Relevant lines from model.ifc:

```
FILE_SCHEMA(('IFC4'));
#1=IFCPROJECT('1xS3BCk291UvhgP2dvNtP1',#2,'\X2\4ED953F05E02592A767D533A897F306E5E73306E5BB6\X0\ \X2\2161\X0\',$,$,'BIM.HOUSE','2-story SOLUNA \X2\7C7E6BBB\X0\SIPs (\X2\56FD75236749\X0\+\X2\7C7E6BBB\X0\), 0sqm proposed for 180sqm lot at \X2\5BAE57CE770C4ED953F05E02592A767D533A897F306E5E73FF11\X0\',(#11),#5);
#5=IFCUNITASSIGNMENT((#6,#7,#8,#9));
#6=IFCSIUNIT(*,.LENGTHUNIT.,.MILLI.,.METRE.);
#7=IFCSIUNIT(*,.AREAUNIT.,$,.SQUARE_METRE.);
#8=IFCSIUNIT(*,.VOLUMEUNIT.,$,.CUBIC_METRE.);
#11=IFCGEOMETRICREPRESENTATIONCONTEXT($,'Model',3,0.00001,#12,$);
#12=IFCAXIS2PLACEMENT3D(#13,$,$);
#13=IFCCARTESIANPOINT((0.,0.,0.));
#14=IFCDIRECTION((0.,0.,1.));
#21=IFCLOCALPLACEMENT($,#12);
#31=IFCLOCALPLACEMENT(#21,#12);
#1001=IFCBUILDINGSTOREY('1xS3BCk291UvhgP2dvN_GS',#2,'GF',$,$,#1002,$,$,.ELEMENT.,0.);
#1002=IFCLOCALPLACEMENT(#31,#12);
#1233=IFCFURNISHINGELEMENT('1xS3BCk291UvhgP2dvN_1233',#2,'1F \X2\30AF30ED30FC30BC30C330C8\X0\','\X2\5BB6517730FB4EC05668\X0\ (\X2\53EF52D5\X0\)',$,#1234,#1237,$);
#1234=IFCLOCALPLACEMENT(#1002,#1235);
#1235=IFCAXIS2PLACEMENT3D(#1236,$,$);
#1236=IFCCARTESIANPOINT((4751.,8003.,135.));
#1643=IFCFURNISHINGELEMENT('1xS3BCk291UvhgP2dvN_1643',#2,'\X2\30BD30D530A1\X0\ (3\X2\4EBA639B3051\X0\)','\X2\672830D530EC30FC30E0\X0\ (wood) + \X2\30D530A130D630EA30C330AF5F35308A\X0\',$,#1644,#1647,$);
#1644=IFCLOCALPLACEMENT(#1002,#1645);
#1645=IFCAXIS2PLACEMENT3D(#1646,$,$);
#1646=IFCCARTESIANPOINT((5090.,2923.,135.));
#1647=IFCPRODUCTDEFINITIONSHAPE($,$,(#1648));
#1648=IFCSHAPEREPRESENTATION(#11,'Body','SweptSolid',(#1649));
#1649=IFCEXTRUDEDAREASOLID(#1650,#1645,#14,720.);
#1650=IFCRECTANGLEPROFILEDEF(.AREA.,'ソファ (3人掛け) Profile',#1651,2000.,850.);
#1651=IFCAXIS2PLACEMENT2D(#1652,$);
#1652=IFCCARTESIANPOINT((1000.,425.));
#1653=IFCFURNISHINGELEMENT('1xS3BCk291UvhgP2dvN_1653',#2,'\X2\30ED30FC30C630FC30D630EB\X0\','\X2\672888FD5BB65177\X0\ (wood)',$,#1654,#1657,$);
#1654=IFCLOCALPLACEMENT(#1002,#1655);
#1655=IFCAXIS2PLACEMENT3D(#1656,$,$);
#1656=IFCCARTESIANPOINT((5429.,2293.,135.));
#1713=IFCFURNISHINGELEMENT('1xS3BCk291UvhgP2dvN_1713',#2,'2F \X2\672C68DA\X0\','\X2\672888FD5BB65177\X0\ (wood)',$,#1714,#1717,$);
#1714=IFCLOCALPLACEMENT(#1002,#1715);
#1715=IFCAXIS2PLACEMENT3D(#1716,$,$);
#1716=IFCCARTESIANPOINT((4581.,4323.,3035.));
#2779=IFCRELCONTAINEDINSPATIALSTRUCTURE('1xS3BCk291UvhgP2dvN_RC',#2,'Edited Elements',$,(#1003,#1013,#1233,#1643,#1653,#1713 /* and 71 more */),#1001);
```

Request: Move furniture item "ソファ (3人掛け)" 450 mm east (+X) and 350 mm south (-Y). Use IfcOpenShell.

```python
import ifcopenshell
import ifcopenshell.api.geometry
import ifcopenshell.util.placement
import ifcopenshell.util.unit

model = ifcopenshell.open("model.ifc")
unit_scale = ifcopenshell.util.unit.calculate_unit_scale(model)

item = model.by_id(1643)
matrix = ifcopenshell.util.placement.get_local_placement(item.ObjectPlacement)
matrix[0, 3] += 0.45 / unit_scale
matrix[1, 3] -= 0.35 / unit_scale
ifcopenshell.api.geometry.edit_object_placement(model, product=item, matrix=matrix, is_si=False)

print(ifcopenshell.util.placement.get_local_placement(item.ObjectPlacement).round(3) + 0.0)

model.write("model_rev.ifc")
```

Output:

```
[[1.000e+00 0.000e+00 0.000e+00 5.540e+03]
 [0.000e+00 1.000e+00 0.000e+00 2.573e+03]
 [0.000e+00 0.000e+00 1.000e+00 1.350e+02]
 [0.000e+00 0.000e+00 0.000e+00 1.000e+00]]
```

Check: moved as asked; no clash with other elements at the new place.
